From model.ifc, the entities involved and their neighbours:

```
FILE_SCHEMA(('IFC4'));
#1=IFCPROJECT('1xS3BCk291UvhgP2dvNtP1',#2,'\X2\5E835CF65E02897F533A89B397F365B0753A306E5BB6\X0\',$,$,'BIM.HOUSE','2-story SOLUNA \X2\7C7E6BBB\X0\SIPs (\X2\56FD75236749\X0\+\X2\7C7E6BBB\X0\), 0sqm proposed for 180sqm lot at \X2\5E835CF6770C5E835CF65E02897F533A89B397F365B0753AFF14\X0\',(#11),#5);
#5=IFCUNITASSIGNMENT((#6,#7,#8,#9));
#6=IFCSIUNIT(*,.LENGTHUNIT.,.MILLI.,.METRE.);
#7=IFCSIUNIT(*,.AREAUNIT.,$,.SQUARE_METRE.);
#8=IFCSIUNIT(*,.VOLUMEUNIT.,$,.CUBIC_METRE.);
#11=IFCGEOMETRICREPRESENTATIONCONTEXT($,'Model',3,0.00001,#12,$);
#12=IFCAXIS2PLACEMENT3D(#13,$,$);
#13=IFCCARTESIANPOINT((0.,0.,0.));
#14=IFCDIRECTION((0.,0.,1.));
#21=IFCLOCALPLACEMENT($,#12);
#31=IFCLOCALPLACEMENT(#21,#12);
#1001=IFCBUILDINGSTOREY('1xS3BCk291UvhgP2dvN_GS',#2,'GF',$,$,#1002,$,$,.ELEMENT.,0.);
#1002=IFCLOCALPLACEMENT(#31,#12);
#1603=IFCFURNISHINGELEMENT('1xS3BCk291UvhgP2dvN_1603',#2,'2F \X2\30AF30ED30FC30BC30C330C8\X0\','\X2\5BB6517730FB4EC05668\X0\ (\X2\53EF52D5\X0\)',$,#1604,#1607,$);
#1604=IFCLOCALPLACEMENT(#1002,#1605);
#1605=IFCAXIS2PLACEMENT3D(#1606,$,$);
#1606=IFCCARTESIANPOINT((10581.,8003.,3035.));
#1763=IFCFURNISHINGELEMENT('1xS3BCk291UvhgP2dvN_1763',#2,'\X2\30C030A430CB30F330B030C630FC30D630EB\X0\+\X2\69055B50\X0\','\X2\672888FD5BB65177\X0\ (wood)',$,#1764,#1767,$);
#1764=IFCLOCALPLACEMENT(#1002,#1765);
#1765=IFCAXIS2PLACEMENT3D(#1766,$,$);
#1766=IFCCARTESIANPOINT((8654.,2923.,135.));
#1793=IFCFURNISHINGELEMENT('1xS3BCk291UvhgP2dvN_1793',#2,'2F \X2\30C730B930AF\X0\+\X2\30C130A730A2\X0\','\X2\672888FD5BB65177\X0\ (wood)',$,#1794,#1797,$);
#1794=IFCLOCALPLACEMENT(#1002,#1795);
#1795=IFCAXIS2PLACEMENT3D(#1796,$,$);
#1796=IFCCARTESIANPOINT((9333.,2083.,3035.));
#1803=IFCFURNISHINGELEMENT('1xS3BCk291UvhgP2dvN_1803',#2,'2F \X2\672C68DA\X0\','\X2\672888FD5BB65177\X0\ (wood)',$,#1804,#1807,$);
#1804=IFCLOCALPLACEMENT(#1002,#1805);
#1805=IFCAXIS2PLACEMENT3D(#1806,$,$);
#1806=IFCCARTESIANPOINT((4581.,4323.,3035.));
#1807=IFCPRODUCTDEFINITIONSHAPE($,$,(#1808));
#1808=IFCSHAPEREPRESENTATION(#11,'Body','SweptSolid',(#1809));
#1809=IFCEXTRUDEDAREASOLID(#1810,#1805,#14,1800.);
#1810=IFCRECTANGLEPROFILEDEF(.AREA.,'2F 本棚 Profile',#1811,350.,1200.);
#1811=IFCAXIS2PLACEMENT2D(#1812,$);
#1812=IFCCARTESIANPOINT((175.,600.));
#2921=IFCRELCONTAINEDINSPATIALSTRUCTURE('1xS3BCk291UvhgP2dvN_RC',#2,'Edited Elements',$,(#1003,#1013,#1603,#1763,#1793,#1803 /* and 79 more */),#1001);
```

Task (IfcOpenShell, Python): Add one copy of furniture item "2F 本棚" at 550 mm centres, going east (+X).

```python
import numpy as np
import ifcopenshell
import ifcopenshell.api.geometry
import ifcopenshell.api.root
import ifcopenshell.util.element
import ifcopenshell.util.placement
import ifcopenshell.util.unit

model = ifcopenshell.open("model.ifc")
unit_scale = ifcopenshell.util.unit.calculate_unit_scale(model)


def reuse_history(source, copy):
    """copy_class also copies each property set's owner history, people and application; keep the originals."""
    for rel in copy.IsDefinedBy:
        if rel.is_a("IfcRelDefinesByProperties") and (history := rel.RelatingPropertyDefinition.OwnerHistory):
            rel.RelatingPropertyDefinition.OwnerHistory = source.OwnerHistory
            ifcopenshell.util.element.remove_deep2(model, history)


source = model.by_guid("1xS3BCk291UvhgP2dvN_1803")
base = ifcopenshell.util.placement.get_local_placement(source.ObjectPlacement)
step = np.array([1.0, 0.0, 0.0]) * 0.55 / unit_scale

for i in range(1, 2):
    copy = ifcopenshell.api.root.copy_class(model, product=source)
    copy.Representation = ifcopenshell.util.element.copy_deep(
        model, source.Representation, exclude=["IfcGeometricRepresentationContext", "IfcRepresentationMap"]
    )
    reuse_history(source, copy)
    matrix = base.copy()
    matrix[:3, 3] += i * step
    print("added at", matrix[:3, 3].round(3) + 0.0)
    ifcopenshell.api.geometry.edit_object_placement(model, product=copy, matrix=matrix, is_si=False)

model.write("model_rev.ifc")
```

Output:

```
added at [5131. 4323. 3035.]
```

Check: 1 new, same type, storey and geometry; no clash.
